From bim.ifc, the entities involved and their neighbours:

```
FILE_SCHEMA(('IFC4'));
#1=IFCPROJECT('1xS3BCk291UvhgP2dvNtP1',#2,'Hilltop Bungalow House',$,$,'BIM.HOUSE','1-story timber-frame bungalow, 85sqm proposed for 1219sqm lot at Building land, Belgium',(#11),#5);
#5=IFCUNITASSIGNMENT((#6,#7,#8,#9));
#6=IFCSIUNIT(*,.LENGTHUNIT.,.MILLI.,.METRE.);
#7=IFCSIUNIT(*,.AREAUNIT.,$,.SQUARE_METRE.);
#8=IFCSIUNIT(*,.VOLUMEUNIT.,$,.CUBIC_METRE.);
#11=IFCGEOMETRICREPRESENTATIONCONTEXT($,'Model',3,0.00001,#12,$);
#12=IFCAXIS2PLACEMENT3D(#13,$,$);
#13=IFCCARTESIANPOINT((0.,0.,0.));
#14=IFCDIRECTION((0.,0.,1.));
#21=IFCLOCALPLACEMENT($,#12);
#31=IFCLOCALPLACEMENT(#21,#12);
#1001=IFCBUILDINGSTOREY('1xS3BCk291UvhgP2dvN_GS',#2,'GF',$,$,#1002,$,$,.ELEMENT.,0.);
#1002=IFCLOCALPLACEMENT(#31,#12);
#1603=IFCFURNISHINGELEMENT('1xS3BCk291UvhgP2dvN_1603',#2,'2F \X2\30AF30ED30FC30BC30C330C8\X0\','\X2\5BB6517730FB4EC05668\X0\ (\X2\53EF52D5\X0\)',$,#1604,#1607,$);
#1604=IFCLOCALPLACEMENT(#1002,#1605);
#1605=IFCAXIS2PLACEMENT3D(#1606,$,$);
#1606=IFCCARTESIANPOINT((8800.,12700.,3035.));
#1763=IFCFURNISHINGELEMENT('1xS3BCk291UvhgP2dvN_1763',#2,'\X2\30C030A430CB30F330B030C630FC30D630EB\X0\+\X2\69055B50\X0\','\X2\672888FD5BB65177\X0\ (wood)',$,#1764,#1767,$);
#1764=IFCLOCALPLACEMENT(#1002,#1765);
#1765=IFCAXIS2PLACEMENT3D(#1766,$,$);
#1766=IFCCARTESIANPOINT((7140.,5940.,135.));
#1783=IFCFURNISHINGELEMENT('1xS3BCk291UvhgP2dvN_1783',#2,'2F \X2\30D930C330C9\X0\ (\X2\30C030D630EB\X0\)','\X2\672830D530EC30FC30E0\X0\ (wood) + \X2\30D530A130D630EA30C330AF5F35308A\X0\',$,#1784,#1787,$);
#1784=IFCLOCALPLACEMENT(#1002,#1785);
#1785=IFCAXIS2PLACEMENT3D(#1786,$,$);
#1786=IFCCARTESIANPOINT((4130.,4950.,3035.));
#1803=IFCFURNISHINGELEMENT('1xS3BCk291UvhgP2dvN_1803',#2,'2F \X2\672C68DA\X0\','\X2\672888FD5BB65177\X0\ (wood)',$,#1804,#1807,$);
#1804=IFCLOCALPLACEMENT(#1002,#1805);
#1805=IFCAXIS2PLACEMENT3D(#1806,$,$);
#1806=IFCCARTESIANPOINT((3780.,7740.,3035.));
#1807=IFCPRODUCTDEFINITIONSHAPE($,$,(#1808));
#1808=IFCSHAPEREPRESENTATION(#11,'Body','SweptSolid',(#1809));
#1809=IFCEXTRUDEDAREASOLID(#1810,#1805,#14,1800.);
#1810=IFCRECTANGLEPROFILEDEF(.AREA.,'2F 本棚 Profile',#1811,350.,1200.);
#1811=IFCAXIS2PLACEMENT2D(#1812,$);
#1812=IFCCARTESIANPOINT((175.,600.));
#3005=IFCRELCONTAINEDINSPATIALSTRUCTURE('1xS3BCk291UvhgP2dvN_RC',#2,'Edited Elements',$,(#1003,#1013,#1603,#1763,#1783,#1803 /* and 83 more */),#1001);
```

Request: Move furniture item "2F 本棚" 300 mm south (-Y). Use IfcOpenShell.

```python
import ifcopenshell
import ifcopenshell.api.geometry
import ifcopenshell.util.placement
import ifcopenshell.util.unit

model = ifcopenshell.open("bim.ifc")
unit_scale = ifcopenshell.util.unit.calculate_unit_scale(model)

item = model.by_guid("1xS3BCk291UvhgP2dvN_1803")
matrix = ifcopenshell.util.placement.get_local_placement(item.ObjectPlacement)
matrix[1, 3] -= 0.3 / unit_scale
ifcopenshell.api.geometry.edit_object_placement(model, product=item, matrix=matrix, is_si=False)

print(ifcopenshell.util.placement.get_local_placement(item.ObjectPlacement).round(3) + 0.0)

model.write("bim_edited.ifc")
```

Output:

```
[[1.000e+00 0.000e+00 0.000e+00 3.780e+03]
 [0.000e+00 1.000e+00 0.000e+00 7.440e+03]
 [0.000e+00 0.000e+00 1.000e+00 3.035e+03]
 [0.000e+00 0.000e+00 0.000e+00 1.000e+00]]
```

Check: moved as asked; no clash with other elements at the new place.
